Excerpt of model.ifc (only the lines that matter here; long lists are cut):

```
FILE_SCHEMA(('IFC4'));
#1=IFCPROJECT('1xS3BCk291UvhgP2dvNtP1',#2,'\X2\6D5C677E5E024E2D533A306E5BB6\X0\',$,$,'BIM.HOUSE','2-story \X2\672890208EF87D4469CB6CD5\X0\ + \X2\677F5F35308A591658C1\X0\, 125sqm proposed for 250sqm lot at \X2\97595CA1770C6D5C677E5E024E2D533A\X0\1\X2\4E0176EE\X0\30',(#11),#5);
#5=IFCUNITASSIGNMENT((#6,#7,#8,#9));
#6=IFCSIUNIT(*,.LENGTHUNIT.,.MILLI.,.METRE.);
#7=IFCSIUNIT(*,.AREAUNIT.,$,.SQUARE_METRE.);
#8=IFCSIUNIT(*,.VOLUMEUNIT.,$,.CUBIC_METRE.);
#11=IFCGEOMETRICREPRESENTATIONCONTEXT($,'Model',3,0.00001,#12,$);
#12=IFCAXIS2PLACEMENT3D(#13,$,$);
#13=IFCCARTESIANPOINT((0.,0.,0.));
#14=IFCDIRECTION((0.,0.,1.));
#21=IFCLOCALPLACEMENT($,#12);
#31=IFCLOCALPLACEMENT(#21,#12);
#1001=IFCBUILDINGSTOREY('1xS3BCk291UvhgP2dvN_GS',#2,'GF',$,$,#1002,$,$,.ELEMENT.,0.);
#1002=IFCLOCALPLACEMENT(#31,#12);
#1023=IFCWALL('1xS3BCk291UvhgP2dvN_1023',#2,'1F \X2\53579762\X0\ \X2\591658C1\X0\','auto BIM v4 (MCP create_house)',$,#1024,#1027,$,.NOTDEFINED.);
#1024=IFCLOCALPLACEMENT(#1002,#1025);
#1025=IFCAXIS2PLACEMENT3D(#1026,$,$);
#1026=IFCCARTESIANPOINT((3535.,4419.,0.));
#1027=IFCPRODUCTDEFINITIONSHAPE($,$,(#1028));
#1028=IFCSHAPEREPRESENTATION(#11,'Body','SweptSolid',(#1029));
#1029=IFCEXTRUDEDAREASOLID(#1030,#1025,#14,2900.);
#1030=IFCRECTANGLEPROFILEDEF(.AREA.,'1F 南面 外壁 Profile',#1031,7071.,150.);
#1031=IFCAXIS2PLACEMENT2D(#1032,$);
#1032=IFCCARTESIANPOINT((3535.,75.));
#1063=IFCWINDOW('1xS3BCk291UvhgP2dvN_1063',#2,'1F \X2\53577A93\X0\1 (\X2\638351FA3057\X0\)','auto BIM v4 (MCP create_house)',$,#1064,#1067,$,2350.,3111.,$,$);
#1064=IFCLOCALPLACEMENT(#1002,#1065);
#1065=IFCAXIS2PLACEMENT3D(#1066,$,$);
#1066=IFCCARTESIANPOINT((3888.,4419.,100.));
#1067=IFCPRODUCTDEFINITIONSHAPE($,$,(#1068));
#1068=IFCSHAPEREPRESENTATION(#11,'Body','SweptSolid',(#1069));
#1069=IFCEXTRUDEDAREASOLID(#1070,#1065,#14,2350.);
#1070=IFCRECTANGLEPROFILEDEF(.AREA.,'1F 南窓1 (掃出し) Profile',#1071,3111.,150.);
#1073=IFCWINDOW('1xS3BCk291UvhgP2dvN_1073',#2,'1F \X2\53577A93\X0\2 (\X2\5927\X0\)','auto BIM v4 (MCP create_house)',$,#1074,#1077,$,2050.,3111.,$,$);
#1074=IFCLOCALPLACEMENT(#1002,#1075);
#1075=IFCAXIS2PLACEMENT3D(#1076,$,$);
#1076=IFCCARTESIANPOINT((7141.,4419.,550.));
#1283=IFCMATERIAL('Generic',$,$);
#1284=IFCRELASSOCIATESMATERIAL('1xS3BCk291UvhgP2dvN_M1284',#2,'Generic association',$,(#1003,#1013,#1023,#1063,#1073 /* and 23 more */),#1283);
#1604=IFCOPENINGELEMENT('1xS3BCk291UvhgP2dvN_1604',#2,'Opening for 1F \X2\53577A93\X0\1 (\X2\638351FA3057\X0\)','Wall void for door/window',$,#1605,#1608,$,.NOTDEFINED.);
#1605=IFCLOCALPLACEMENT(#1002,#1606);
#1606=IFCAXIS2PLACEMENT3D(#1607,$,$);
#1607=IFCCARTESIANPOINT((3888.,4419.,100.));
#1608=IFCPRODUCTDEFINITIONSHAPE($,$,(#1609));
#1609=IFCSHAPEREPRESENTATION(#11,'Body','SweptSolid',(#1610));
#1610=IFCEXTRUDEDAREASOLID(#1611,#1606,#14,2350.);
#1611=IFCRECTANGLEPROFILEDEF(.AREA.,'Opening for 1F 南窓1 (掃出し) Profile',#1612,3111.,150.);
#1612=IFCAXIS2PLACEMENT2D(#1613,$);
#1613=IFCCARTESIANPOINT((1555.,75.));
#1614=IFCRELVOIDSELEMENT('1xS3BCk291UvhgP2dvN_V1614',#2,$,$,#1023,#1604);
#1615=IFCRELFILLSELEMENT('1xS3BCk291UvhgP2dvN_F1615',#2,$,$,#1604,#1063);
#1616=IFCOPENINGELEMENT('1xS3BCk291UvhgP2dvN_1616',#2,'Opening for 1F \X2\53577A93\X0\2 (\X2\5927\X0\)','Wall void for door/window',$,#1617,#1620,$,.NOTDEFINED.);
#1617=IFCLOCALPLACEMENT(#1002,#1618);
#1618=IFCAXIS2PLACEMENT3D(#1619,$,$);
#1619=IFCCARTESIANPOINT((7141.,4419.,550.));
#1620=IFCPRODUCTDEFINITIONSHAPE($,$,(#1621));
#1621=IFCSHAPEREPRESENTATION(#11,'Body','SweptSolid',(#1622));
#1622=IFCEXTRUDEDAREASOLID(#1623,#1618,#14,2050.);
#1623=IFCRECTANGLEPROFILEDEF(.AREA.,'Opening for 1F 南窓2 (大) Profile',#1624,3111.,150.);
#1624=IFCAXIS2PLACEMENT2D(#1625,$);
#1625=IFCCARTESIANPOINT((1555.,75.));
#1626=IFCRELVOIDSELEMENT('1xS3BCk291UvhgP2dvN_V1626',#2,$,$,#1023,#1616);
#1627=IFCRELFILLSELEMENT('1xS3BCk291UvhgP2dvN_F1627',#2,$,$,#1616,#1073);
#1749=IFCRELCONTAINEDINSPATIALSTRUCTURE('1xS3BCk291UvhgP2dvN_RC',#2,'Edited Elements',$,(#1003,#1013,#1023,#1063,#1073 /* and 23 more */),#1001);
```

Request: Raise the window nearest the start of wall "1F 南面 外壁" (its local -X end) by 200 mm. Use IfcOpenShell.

```python
import numpy as np
import ifcopenshell
import ifcopenshell.api.geometry
import ifcopenshell.util.placement
import ifcopenshell.util.unit

model = ifcopenshell.open("model.ifc")
unit_scale = ifcopenshell.util.unit.calculate_unit_scale(model)

window = model.by_guid("1xS3BCk291UvhgP2dvN_1063")
opening = window.FillsVoids[0].RelatingOpeningElement
dz = 0.2 / unit_scale

shift = np.array([0.0, 0.0, dz])
# The window is not placed relative to its opening, so move both.
for product in (opening, window):
    matrix = ifcopenshell.util.placement.get_local_placement(product.ObjectPlacement)
    matrix[:3, 3] += shift
    ifcopenshell.api.geometry.edit_object_placement(model, product=product, matrix=matrix, is_si=False)

print(f"moved by {dz * unit_scale:+.3f} m")

model.write("model-out.ifc")
```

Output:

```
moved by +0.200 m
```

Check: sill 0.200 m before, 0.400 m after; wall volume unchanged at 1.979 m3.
